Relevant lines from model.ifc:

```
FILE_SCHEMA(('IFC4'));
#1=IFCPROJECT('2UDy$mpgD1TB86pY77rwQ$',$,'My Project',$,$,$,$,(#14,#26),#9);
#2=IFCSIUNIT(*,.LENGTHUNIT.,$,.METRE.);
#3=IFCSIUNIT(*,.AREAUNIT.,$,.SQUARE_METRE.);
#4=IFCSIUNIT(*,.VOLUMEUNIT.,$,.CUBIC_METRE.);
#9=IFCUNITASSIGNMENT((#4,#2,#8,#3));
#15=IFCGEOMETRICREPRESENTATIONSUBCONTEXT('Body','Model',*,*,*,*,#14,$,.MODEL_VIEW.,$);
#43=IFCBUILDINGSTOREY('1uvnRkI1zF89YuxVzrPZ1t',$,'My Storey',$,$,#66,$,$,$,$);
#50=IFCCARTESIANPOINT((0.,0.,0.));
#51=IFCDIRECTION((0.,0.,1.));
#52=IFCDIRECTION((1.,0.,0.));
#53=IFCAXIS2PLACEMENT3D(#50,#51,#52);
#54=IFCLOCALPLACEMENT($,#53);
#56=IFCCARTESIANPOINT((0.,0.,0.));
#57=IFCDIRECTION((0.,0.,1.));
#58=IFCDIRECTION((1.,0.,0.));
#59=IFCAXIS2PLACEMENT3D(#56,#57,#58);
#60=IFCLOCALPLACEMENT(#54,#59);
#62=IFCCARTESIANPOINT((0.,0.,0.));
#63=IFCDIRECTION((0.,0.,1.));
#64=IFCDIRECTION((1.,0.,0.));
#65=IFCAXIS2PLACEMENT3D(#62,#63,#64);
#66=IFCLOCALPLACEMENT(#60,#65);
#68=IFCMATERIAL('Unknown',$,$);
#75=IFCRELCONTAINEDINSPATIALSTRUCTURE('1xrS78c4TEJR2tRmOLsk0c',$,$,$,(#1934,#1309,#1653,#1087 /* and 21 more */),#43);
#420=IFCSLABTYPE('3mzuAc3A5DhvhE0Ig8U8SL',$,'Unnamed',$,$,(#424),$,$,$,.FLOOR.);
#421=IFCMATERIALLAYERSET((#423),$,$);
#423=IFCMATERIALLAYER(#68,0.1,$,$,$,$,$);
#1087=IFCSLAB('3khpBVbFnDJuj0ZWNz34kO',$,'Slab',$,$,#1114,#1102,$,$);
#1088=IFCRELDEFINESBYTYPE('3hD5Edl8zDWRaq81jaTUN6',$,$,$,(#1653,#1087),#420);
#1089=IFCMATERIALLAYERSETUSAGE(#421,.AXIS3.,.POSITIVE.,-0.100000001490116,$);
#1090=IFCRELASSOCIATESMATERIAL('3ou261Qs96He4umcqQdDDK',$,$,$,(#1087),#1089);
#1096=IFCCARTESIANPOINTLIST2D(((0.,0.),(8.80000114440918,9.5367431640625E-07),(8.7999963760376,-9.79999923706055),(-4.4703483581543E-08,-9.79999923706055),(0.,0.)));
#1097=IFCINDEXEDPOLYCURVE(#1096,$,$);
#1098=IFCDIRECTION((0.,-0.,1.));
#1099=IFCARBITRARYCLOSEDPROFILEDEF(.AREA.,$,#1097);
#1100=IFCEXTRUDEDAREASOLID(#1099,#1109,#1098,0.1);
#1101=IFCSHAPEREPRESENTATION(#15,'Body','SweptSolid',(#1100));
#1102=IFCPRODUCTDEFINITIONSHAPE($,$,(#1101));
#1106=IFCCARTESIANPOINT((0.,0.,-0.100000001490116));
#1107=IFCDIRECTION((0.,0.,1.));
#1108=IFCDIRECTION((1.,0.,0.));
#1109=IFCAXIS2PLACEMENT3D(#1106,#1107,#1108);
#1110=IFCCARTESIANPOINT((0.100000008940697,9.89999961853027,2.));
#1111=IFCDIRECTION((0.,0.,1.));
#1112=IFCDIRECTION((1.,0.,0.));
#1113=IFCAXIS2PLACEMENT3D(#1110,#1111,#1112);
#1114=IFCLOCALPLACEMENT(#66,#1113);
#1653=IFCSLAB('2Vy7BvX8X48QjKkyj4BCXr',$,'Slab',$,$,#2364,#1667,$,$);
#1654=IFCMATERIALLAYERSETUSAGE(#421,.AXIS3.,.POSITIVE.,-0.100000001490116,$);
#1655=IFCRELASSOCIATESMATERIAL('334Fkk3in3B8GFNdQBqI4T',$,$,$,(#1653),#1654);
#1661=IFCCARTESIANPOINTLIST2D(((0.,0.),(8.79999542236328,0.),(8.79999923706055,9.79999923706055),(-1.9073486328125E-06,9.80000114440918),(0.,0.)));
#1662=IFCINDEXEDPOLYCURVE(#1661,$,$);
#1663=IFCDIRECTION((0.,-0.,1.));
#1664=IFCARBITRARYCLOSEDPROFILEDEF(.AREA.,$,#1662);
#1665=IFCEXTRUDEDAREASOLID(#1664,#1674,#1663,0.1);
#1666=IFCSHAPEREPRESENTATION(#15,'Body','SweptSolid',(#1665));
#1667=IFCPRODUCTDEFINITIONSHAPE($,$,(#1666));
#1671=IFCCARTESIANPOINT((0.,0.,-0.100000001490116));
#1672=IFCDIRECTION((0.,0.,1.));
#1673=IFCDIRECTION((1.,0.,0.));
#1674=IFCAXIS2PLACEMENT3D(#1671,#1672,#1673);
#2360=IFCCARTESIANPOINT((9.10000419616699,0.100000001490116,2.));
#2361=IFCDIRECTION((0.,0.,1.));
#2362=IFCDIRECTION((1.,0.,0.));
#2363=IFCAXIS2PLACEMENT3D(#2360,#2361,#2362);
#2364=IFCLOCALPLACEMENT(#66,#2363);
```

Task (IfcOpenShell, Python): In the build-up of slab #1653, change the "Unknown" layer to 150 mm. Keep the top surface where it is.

```python
import ifcopenshell
import ifcopenshell.util.element
import ifcopenshell.util.representation

model = ifcopenshell.open("model.ifc")

layer_set = model.by_id(421)
layer = next(l for l in layer_set.MaterialLayers if l.Material and l.Material.Name == "Unknown")
change = 0.15 - layer.LayerThickness
layer.LayerThickness += change

# The layer set is shared, so every slab that uses it gets the new thickness.
slabs = [e for e in ifcopenshell.util.element.get_elements_by_material(model, layer_set) if e.is_a("IfcSlab")]
for slab in sorted(slabs, key=lambda e: e.id()):
    body = ifcopenshell.util.representation.get_representation(slab, "Model", "Body")
    solid = body.Items[0]
    old_depth = solid.Depth
    solid.Depth += change
    # Extruded upwards: lower the start of the extrusion so the top stays.
    x, y, z = solid.Position.Location.Coordinates
    solid.Position.Location = model.createIfcCartesianPoint((x, y, z - change))
    print(slab.id(), f"{old_depth:g} -> {solid.Depth:g}")

# The layers are counted up from the underside, which has moved.
for usage in {ifcopenshell.util.element.get_material(slab) for slab in slabs}:
    usage.OffsetFromReferenceLine -= change

model.write("model-out.ifc")
```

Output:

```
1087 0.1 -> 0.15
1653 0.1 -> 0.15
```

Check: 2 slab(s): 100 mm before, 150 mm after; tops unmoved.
